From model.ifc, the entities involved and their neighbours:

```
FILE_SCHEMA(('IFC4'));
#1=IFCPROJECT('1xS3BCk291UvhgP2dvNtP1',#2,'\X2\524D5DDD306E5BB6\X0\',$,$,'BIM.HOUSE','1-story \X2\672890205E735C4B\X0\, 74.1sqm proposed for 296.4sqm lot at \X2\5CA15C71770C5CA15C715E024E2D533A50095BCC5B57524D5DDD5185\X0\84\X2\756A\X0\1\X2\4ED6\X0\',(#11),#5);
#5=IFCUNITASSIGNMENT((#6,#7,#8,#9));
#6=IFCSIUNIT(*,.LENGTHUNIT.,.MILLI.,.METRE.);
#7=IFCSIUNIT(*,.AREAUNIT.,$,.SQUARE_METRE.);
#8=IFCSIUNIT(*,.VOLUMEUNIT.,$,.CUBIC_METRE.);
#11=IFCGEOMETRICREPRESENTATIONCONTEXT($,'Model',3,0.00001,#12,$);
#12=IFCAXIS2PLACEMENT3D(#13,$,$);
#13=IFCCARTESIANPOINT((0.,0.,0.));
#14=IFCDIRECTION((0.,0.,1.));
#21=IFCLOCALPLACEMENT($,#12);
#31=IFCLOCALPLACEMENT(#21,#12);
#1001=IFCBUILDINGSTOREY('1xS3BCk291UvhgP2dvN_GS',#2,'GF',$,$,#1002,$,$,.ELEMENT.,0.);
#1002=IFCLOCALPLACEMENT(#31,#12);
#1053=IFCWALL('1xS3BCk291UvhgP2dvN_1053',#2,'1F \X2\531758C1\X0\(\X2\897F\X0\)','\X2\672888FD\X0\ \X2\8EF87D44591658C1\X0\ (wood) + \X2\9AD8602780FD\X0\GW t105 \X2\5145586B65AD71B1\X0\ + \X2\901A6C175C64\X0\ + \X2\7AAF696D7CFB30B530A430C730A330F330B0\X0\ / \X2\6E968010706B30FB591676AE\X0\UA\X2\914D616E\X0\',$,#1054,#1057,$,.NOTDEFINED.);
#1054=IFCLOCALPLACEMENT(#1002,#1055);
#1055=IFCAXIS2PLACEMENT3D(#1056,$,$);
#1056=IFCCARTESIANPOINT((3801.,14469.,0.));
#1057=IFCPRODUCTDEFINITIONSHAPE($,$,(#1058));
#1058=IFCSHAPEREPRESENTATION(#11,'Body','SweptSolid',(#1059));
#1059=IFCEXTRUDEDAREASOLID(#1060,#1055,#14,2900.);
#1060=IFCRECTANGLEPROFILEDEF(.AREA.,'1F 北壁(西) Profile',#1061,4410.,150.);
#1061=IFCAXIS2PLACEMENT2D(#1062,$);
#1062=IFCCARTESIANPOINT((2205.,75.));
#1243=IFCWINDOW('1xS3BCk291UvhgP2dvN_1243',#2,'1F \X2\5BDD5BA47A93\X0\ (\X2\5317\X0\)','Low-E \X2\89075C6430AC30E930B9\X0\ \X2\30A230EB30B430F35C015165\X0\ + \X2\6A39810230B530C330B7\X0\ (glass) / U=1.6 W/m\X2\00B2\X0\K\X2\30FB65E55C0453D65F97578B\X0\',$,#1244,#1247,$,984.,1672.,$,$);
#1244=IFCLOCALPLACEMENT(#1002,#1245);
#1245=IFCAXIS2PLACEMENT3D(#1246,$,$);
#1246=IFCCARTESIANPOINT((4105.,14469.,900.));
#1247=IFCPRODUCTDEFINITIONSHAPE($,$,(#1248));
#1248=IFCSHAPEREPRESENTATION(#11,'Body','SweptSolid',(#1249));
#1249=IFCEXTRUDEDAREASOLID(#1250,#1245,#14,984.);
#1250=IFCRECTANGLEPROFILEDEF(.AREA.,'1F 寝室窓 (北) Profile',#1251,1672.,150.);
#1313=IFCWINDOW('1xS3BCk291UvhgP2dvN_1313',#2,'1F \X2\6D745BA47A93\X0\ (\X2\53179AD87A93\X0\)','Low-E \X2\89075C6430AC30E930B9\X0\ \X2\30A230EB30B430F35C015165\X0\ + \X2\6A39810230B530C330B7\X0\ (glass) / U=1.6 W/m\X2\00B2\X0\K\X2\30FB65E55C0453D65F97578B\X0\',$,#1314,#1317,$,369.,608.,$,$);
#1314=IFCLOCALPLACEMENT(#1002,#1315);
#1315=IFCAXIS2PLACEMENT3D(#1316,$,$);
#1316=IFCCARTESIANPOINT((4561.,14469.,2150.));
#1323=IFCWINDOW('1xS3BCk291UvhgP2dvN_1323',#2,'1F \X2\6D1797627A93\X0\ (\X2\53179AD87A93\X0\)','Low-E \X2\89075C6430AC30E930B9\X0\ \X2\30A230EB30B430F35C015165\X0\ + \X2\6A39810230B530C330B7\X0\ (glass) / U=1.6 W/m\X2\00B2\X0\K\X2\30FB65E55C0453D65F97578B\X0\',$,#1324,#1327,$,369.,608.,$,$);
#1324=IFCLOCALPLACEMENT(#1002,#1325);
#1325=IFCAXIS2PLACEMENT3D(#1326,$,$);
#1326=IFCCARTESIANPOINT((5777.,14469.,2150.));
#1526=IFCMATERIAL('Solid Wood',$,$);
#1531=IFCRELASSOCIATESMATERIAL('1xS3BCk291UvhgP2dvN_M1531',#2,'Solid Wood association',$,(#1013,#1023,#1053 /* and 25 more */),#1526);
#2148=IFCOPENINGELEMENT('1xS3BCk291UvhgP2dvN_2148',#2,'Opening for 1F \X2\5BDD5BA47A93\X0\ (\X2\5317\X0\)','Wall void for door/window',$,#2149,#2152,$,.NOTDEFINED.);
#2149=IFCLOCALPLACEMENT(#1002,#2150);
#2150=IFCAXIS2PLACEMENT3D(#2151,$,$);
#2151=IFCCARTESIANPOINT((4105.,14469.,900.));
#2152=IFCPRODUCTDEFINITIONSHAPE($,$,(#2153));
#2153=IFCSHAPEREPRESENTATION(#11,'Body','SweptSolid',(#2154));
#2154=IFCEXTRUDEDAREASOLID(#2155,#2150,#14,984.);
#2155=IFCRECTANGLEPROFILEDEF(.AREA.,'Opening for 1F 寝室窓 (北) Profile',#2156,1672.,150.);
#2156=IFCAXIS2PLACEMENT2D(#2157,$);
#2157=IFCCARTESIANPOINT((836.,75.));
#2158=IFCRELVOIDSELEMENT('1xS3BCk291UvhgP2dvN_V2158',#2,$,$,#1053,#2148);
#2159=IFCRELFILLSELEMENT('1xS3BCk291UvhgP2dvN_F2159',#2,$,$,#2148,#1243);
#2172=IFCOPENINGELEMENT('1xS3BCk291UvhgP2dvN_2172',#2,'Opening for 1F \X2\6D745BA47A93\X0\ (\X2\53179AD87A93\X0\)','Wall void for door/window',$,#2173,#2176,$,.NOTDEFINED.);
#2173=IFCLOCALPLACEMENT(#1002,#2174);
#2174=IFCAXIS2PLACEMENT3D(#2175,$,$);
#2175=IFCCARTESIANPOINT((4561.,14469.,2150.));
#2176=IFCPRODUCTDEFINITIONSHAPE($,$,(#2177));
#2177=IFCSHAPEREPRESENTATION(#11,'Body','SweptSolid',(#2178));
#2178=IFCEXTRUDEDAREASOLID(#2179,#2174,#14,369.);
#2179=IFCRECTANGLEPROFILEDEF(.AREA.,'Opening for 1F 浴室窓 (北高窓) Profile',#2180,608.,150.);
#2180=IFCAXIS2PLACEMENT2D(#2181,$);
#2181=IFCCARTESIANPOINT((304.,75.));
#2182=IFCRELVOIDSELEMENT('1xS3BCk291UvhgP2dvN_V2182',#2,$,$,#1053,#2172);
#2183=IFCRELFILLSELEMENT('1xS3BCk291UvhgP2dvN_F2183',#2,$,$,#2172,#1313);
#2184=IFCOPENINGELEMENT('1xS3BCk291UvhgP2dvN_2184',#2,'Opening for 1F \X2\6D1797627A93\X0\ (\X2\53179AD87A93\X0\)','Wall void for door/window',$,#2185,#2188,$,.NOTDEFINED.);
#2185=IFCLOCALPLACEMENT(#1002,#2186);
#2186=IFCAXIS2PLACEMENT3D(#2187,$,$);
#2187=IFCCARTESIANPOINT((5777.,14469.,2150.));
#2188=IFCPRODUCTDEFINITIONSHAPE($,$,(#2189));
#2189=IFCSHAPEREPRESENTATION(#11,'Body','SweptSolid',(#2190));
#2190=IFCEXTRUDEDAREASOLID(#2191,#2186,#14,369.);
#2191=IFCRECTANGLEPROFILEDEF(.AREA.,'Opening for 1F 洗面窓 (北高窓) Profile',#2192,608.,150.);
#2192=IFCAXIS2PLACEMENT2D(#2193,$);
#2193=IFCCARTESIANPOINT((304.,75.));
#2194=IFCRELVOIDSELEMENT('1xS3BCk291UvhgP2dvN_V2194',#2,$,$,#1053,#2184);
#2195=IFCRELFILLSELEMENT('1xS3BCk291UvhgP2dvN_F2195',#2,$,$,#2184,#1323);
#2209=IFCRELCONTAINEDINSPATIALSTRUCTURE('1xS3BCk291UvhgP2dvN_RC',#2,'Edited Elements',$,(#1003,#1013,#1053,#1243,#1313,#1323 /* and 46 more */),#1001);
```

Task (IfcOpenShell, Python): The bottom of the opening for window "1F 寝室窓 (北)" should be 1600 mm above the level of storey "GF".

```python
import numpy as np
import ifcopenshell
import ifcopenshell.api.geometry
import ifcopenshell.geom
import ifcopenshell.util.element
import ifcopenshell.util.placement
import ifcopenshell.util.shape
import ifcopenshell.util.unit

model = ifcopenshell.open("model.ifc")
unit_scale = ifcopenshell.util.unit.calculate_unit_scale(model)

window = model.by_id(1243)
opening = window.FillsVoids[0].RelatingOpeningElement
storey = ifcopenshell.util.element.get_container(window, ifc_class="IfcBuildingStorey")
level = ifcopenshell.util.placement.get_local_placement(storey.ObjectPlacement)[2, 3]

# The opening's origin need not be at the sill, so measure its lowest point.
shape = ifcopenshell.geom.create_shape(ifcopenshell.geom.settings(), opening)
bottom = ifcopenshell.util.shape.get_shape_bottom_elevation(shape, shape.geometry) / unit_scale
dz = level + 1600.0 - bottom

shift = np.array([0.0, 0.0, dz])
# The window is not placed relative to its opening, so move both.
for product in (opening, window):
    matrix = ifcopenshell.util.placement.get_local_placement(product.ObjectPlacement)
    matrix[:3, 3] += shift
    ifcopenshell.api.geometry.edit_object_placement(model, product=product, matrix=matrix, is_si=False)

print(f"moved by {dz * unit_scale:+.3f} m")

model.write("model_updated.ifc")
```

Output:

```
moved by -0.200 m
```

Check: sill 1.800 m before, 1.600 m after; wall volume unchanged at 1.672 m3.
